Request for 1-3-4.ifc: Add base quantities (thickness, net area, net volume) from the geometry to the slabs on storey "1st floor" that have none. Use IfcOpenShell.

First a look at what the model holds.

```python
import ifcopenshell
import ifcopenshell.util.element
import ifcopenshell.util.unit

model = ifcopenshell.open("1-3-4.ifc")
print(model.schema)
for unit_type in ("LENGTHUNIT", "AREAUNIT", "VOLUMEUNIT"):
    print(unit_type, ifcopenshell.util.unit.calculate_unit_scale(model, unit_type))
storey = next(s for s in model.by_type("IfcBuildingStorey") if s.Name == "1st floor")
slabs = [e for e in ifcopenshell.util.element.get_decomposition(storey) if e.is_a("IfcSlab")]
for e in sorted(slabs, key=lambda e: e.id()):
    print(e.id(), e.is_a(), e.Name, list(ifcopenshell.util.element.get_psets(e, qtos_only=True)), sep=" | ")
```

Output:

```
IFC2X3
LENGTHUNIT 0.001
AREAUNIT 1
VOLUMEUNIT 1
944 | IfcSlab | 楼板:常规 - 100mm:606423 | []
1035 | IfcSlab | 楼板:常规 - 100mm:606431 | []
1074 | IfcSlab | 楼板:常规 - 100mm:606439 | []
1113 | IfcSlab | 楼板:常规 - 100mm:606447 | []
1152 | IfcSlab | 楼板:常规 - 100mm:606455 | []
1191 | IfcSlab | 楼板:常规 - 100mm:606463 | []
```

```python
import ifcopenshell
import ifcopenshell.api.pset
import ifcopenshell.geom
import ifcopenshell.util.element
import ifcopenshell.util.shape
import ifcopenshell.util.unit

model = ifcopenshell.open("1-3-4.ifc")
unit_scale = ifcopenshell.util.unit.calculate_unit_scale(model)
area_scale = ifcopenshell.util.unit.calculate_unit_scale(model, "AREAUNIT")
volume_scale = ifcopenshell.util.unit.calculate_unit_scale(model, "VOLUMEUNIT")
settings = ifcopenshell.geom.settings()

storey = next(s for s in model.by_type("IfcBuildingStorey") if s.Name == "1st floor")
slabs = [e for e in ifcopenshell.util.element.get_decomposition(storey) if e.is_a("IfcSlab")]

for e in sorted(slabs, key=lambda e: e.id()):
    if ifcopenshell.util.element.get_psets(e, qtos_only=True, should_inherit=False):
        continue
    # Geometry comes back in metres, in the element's own axes.
    shape = ifcopenshell.geom.create_shape(settings, e)
    values = {
        "Width": ifcopenshell.util.shape.get_z(shape.geometry) / unit_scale,
        "NetArea": ifcopenshell.util.shape.get_footprint_area(shape.geometry) / area_scale,
        "NetVolume": ifcopenshell.util.shape.get_volume(shape.geometry) / volume_scale,
    }
    qto = ifcopenshell.api.pset.add_qto(model, product=e, name="BaseQuantities")
    ifcopenshell.api.pset.edit_qto(model, qto=qto, properties=values)
    print(e.id(), {k: round(v, 3) for k, v in values.items()})

model.write("1-3-4_rev.ifc")
```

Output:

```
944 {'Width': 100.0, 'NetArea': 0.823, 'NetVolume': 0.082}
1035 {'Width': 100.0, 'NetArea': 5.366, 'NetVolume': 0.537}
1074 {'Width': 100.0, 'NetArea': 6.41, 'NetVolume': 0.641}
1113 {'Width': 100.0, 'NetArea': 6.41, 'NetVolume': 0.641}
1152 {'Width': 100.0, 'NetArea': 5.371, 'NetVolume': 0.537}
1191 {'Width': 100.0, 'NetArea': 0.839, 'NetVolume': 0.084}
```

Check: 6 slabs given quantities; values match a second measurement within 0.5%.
